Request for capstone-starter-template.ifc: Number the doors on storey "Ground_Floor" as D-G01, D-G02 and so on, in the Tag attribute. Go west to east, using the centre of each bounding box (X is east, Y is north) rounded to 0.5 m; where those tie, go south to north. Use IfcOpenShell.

First a look at what the model holds.

```python
import ifcopenshell
import ifcopenshell.util.element
import ifcopenshell.util.placement

model = ifcopenshell.open("capstone-starter-template.ifc")
print(model.schema)
storey = next(s for s in model.by_type("IfcBuildingStorey") if s.Name == "Ground_Floor")
doors = [e for e in ifcopenshell.util.element.get_decomposition(storey) if e.is_a("IfcDoor")]
for e in sorted(doors, key=lambda e: e.id()):
    origin = ifcopenshell.util.placement.get_local_placement(e.ObjectPlacement)[:3, 3]
    print(e.id(), e.Tag, e.Name, origin.round(2) + 0.0, sep=" | ")
```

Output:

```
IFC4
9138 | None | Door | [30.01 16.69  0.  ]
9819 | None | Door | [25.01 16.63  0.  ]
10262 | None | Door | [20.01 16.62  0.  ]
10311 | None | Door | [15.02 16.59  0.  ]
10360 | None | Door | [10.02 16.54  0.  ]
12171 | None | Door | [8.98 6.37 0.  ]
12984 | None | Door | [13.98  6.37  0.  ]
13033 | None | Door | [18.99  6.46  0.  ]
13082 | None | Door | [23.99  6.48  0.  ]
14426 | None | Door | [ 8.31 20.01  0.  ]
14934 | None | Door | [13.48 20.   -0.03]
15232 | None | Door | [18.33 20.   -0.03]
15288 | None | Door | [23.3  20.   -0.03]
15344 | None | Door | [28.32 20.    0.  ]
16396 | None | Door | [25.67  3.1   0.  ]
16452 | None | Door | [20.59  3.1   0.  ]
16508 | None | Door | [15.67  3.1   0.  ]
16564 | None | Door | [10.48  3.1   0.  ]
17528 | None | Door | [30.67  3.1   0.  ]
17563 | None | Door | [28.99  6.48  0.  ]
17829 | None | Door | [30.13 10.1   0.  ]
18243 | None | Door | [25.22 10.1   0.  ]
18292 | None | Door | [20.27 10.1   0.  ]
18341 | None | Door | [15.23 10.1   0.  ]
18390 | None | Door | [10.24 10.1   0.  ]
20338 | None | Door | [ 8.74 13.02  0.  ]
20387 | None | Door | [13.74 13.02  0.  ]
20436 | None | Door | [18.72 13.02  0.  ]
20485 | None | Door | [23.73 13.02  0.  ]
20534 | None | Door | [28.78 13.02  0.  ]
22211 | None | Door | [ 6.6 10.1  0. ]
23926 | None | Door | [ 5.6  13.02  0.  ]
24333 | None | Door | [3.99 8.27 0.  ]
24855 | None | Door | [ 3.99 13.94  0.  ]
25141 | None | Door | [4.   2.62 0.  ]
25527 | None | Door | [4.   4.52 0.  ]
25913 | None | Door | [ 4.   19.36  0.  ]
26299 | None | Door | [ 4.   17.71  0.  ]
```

```python
import ifcopenshell
import ifcopenshell.geom
import ifcopenshell.util.element
import ifcopenshell.util.shape

model = ifcopenshell.open("capstone-starter-template.ifc")
settings = ifcopenshell.geom.settings()
settings.set("use-world-coords", True)


def centre(element):
    shape = ifcopenshell.geom.create_shape(settings, element)
    return ifcopenshell.util.shape.get_bbox_centroid(shape.geometry)


storey = next(s for s in model.by_type("IfcBuildingStorey") if s.Name == "Ground_Floor")
doors = [e for e in ifcopenshell.util.element.get_decomposition(storey) if e.is_a("IfcDoor")]

# Insertion points can sit at a corner or the storey origin, so sort by the geometry (in metres).
centres = {e: centre(e) for e in doors}
doors.sort(key=lambda e: (round(centres[e][0] / 0.5), centres[e][1]))

for i, e in enumerate(doors, start=1):
    number = f"D-G{i:02d}"
    e.Tag = number
    print(e.id(), number)

model.write("capstone-starter-template_updated.ifc")
```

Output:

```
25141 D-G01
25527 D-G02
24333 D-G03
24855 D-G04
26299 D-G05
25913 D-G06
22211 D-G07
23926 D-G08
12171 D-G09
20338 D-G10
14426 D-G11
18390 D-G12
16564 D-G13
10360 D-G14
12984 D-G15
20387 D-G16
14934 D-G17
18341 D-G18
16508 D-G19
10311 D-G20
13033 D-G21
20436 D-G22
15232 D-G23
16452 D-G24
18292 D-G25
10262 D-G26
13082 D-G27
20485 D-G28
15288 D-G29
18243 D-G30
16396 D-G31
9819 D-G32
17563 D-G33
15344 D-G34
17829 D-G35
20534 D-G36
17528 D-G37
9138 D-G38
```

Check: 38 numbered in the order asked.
